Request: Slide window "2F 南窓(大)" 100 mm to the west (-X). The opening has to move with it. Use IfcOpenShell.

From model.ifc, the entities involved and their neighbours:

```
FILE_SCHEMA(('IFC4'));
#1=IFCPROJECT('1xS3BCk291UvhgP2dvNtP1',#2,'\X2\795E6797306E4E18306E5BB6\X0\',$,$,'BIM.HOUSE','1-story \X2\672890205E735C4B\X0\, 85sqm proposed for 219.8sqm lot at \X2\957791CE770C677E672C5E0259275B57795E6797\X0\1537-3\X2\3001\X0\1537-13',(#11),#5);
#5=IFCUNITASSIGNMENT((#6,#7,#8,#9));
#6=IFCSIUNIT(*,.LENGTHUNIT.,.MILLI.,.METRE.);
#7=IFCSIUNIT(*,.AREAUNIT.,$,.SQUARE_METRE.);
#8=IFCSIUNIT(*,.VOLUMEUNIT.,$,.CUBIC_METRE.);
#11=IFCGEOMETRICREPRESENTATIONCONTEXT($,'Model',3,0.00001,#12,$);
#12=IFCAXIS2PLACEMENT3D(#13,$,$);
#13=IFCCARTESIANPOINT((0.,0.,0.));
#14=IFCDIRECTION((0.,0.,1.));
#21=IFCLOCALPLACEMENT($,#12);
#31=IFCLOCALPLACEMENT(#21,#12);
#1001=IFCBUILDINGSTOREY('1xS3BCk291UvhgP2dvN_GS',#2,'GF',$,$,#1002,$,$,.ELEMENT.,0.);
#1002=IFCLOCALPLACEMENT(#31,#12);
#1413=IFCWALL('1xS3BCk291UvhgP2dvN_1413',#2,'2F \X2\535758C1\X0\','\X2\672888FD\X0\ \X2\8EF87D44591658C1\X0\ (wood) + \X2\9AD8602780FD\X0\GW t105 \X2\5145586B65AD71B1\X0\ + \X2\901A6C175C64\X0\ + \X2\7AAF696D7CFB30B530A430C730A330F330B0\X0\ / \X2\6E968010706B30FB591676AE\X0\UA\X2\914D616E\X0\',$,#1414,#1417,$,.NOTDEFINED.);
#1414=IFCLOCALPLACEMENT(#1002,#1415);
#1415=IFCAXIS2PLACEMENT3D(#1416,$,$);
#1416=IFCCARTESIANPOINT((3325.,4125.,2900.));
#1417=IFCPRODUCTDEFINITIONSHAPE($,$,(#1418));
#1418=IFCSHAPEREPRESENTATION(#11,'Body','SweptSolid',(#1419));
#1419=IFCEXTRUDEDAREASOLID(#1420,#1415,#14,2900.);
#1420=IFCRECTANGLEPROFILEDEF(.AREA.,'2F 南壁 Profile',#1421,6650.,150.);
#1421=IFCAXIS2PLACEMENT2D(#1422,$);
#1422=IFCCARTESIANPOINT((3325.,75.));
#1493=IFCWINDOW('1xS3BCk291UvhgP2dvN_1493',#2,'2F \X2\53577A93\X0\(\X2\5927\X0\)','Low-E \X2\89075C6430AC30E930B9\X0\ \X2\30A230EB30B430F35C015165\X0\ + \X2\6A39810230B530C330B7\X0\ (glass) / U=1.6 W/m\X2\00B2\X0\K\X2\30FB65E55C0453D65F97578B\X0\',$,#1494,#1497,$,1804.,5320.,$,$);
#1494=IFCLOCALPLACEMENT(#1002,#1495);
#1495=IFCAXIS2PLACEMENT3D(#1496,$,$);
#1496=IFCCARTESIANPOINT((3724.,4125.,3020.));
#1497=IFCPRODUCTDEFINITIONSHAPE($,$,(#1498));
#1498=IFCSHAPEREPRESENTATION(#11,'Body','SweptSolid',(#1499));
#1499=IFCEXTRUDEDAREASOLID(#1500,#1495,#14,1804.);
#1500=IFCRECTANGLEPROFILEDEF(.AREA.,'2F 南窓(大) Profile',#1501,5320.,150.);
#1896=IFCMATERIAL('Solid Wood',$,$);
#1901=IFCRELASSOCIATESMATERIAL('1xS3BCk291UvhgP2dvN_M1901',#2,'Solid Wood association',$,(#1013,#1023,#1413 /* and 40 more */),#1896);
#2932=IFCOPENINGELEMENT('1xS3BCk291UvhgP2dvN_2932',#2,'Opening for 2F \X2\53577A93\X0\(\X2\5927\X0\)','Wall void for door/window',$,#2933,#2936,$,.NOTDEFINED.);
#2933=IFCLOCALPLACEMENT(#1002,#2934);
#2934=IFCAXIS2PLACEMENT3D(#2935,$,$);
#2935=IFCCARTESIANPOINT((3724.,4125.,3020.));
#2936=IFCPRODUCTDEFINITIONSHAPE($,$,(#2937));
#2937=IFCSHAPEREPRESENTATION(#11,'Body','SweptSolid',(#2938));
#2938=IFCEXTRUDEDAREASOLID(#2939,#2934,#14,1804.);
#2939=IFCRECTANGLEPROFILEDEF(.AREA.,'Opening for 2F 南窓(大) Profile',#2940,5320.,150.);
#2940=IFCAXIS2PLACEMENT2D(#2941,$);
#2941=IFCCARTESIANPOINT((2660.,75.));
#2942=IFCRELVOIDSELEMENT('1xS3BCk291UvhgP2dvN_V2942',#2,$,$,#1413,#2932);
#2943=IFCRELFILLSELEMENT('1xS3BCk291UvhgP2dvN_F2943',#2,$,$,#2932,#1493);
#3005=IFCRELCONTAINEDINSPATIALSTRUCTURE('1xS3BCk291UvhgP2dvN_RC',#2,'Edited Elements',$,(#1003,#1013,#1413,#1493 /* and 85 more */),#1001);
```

```python
import ifcopenshell
import ifcopenshell.api.geometry
import ifcopenshell.util.placement

model = ifcopenshell.open("model.ifc")

window = model.by_id(1493)
opening = window.FillsVoids[0].RelatingOpeningElement
wall = opening.VoidsElements[0].RelatingBuildingElement

wall_matrix = ifcopenshell.util.placement.get_local_placement(wall.ObjectPlacement)
shift = wall_matrix[:3, 0] * -100.0
before = ifcopenshell.util.placement.get_local_placement(window.ObjectPlacement)[:3, 3].copy()

# The window is not placed relative to its opening, so move both.
for product in (opening, window):
    matrix = ifcopenshell.util.placement.get_local_placement(product.ObjectPlacement)
    matrix[:3, 3] += shift
    ifcopenshell.api.geometry.edit_object_placement(model, product=product, matrix=matrix, is_si=False)

after = ifcopenshell.util.placement.get_local_placement(window.ObjectPlacement)[:3, 3]
print("window moved by", (after - before).round(3) + 0.0)

model.write("model_rev.ifc")
```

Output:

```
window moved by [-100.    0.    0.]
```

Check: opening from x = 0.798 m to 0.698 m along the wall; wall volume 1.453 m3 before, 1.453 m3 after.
